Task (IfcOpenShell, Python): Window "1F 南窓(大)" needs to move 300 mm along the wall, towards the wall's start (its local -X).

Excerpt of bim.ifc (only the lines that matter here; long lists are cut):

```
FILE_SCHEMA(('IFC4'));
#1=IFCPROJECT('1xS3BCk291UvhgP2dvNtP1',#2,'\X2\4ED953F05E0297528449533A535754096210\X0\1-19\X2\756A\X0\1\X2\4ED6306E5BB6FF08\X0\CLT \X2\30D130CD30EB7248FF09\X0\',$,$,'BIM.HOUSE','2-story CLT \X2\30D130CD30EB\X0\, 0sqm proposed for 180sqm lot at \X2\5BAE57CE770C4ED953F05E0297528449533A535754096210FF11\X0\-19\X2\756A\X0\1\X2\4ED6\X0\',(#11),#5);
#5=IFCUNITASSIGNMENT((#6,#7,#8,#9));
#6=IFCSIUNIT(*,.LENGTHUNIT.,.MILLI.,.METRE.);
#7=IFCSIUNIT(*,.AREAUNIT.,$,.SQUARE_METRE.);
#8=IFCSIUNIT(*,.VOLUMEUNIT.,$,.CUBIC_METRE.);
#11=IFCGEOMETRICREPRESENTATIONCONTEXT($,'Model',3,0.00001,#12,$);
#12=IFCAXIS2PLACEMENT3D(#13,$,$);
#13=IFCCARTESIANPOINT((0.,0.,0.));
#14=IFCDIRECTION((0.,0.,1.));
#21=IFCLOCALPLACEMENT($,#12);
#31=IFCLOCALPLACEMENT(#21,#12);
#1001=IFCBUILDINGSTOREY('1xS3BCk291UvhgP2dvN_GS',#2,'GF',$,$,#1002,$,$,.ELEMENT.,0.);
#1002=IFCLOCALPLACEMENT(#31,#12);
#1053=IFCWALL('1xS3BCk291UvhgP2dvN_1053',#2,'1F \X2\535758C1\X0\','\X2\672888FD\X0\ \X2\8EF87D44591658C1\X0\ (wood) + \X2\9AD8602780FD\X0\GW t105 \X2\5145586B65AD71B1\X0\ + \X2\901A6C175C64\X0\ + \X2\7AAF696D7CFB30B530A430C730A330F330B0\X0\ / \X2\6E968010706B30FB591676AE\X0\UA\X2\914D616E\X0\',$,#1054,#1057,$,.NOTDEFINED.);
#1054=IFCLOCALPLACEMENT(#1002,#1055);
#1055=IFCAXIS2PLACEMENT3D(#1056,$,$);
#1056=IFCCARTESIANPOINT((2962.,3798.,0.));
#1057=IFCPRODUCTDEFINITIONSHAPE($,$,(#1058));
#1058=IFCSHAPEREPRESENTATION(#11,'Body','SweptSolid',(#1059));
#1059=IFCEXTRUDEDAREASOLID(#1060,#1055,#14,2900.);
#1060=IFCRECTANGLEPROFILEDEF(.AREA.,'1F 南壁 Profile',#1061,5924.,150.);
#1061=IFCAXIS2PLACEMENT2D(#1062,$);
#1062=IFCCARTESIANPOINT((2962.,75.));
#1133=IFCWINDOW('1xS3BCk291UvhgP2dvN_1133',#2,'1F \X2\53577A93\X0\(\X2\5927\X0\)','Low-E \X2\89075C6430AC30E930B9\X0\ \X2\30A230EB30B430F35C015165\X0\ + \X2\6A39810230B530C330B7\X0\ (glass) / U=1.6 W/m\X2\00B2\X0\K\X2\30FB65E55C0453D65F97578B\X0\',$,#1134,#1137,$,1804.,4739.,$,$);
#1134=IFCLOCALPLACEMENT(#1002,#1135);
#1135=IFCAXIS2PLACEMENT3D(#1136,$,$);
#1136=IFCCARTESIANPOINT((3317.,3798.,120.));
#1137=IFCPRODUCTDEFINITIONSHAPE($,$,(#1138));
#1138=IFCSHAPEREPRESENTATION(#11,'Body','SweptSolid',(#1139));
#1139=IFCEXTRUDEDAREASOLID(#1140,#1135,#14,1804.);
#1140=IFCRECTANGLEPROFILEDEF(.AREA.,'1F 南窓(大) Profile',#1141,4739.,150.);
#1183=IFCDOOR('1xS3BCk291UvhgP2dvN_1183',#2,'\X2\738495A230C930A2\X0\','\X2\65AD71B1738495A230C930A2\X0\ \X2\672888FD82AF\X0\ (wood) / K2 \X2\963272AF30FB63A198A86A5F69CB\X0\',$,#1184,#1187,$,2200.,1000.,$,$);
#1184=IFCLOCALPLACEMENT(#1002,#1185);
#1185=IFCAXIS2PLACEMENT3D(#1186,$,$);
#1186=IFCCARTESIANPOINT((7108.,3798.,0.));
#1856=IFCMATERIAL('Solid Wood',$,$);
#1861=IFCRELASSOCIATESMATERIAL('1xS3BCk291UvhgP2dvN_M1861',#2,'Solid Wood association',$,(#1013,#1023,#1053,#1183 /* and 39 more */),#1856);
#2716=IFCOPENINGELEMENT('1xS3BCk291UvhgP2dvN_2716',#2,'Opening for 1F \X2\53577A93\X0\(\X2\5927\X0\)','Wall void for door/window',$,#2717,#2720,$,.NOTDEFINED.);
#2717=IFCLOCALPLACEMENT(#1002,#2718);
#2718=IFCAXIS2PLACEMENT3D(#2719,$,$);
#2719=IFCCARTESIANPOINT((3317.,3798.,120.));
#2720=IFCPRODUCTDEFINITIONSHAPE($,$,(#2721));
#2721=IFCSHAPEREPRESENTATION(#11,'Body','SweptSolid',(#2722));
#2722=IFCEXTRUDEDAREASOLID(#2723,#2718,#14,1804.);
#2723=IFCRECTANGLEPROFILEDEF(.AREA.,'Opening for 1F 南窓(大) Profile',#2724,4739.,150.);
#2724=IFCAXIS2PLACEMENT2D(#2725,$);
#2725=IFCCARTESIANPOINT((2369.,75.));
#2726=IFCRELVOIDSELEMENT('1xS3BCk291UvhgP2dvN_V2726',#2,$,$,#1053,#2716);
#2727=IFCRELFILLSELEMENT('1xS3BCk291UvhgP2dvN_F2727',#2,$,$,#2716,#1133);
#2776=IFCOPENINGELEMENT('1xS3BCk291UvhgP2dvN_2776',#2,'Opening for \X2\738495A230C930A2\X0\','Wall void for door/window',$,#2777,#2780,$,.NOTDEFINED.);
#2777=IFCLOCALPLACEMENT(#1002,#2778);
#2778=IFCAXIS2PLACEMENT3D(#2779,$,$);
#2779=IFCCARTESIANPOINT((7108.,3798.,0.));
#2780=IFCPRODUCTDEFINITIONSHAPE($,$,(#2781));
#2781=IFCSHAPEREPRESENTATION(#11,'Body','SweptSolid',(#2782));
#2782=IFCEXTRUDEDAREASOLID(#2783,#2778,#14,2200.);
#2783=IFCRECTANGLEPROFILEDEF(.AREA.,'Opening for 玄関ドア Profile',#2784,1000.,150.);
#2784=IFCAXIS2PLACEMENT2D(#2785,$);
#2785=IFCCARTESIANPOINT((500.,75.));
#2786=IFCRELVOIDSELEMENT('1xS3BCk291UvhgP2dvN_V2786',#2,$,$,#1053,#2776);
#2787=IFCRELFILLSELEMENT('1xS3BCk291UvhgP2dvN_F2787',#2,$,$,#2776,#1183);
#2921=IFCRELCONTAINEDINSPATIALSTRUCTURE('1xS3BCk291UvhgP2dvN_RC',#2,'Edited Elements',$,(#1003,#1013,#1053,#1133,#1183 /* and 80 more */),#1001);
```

```python
import ifcopenshell
import ifcopenshell.api.geometry
import ifcopenshell.util.placement
import ifcopenshell.util.unit

model = ifcopenshell.open("bim.ifc")
unit_scale = ifcopenshell.util.unit.calculate_unit_scale(model)

window = model.by_guid("1xS3BCk291UvhgP2dvN_1133")
opening = window.FillsVoids[0].RelatingOpeningElement
wall = opening.VoidsElements[0].RelatingBuildingElement

wall_matrix = ifcopenshell.util.placement.get_local_placement(wall.ObjectPlacement)
shift = wall_matrix[:3, 0] * -0.3 / unit_scale
before = ifcopenshell.util.placement.get_local_placement(window.ObjectPlacement)[:3, 3].copy()

# The window is not placed relative to its opening, so move both.
for product in (opening, window):
    matrix = ifcopenshell.util.placement.get_local_placement(product.ObjectPlacement)
    matrix[:3, 3] += shift
    ifcopenshell.api.geometry.edit_object_placement(model, product=product, matrix=matrix, is_si=False)

after = ifcopenshell.util.placement.get_local_placement(window.ObjectPlacement)[:3, 3]
print("window moved by", (after - before).round(3) + 0.0)

model.write("bim_rev.ifc")
```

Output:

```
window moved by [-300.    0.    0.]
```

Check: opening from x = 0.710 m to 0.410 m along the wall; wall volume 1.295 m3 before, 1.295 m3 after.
